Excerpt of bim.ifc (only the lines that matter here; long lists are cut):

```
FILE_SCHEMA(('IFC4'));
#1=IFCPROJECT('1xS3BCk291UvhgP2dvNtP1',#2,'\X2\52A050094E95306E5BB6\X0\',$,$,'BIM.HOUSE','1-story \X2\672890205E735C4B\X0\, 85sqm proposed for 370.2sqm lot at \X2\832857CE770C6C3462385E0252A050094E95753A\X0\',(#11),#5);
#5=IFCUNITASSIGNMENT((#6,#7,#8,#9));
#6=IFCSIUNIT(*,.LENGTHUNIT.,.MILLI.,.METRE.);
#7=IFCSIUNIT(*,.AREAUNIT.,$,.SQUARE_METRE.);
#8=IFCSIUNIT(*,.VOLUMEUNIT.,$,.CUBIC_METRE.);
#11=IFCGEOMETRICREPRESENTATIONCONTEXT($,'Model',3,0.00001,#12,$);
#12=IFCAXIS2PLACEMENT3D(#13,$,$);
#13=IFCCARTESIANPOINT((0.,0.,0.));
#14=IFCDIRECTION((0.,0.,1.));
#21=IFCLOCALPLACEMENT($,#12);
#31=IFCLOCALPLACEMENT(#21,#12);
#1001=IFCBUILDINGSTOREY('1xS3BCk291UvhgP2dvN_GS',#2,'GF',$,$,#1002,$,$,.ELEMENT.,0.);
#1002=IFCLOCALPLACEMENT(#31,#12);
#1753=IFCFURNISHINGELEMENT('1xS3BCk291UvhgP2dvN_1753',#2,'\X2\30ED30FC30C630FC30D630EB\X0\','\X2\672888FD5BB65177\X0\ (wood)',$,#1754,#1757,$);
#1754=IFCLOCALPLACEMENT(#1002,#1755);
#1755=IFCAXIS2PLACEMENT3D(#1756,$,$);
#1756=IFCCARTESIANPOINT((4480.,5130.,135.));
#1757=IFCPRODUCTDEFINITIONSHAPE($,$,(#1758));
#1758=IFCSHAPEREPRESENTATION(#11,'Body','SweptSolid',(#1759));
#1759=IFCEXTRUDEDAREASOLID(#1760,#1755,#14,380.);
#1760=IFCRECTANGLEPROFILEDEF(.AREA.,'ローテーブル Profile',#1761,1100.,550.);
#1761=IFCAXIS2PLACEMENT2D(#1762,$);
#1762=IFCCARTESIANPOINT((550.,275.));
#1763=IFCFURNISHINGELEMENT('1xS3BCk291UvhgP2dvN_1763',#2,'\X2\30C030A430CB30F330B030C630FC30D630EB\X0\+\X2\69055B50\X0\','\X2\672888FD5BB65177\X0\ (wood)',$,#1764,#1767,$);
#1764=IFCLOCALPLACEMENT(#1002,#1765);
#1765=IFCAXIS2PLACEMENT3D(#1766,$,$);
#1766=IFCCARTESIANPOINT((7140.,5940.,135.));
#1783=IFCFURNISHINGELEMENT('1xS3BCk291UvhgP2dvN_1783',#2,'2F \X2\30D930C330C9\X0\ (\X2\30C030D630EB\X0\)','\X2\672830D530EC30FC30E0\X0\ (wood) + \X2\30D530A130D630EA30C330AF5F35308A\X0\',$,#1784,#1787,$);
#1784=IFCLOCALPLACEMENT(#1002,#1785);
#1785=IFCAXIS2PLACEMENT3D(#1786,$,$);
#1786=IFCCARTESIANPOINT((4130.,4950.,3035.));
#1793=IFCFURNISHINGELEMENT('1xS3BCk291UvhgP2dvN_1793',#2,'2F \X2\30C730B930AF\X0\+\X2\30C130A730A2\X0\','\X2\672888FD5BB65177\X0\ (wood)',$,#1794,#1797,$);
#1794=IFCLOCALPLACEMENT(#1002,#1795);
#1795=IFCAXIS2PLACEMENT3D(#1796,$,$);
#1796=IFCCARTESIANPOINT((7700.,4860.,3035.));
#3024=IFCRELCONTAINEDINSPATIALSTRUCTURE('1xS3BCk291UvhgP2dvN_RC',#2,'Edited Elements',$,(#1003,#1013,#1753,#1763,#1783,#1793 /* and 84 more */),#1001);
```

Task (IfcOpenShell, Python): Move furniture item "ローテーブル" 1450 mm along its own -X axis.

```python
import ifcopenshell
import ifcopenshell.api.geometry
import ifcopenshell.util.placement
import ifcopenshell.util.unit

model = ifcopenshell.open("bim.ifc")
unit_scale = ifcopenshell.util.unit.calculate_unit_scale(model)

item = model.by_guid("1xS3BCk291UvhgP2dvN_1753")
matrix = ifcopenshell.util.placement.get_local_placement(item.ObjectPlacement)
matrix[:3, 3] -= matrix[:3, 0] * 1.45 / unit_scale
ifcopenshell.api.geometry.edit_object_placement(model, product=item, matrix=matrix, is_si=False)

print(ifcopenshell.util.placement.get_local_placement(item.ObjectPlacement).round(3) + 0.0)

model.write("bim_updated.ifc")
```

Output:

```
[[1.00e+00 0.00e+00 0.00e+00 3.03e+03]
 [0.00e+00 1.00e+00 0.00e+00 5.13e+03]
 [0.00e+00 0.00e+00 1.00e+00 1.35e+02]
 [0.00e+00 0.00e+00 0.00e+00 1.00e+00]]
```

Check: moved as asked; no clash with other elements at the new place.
